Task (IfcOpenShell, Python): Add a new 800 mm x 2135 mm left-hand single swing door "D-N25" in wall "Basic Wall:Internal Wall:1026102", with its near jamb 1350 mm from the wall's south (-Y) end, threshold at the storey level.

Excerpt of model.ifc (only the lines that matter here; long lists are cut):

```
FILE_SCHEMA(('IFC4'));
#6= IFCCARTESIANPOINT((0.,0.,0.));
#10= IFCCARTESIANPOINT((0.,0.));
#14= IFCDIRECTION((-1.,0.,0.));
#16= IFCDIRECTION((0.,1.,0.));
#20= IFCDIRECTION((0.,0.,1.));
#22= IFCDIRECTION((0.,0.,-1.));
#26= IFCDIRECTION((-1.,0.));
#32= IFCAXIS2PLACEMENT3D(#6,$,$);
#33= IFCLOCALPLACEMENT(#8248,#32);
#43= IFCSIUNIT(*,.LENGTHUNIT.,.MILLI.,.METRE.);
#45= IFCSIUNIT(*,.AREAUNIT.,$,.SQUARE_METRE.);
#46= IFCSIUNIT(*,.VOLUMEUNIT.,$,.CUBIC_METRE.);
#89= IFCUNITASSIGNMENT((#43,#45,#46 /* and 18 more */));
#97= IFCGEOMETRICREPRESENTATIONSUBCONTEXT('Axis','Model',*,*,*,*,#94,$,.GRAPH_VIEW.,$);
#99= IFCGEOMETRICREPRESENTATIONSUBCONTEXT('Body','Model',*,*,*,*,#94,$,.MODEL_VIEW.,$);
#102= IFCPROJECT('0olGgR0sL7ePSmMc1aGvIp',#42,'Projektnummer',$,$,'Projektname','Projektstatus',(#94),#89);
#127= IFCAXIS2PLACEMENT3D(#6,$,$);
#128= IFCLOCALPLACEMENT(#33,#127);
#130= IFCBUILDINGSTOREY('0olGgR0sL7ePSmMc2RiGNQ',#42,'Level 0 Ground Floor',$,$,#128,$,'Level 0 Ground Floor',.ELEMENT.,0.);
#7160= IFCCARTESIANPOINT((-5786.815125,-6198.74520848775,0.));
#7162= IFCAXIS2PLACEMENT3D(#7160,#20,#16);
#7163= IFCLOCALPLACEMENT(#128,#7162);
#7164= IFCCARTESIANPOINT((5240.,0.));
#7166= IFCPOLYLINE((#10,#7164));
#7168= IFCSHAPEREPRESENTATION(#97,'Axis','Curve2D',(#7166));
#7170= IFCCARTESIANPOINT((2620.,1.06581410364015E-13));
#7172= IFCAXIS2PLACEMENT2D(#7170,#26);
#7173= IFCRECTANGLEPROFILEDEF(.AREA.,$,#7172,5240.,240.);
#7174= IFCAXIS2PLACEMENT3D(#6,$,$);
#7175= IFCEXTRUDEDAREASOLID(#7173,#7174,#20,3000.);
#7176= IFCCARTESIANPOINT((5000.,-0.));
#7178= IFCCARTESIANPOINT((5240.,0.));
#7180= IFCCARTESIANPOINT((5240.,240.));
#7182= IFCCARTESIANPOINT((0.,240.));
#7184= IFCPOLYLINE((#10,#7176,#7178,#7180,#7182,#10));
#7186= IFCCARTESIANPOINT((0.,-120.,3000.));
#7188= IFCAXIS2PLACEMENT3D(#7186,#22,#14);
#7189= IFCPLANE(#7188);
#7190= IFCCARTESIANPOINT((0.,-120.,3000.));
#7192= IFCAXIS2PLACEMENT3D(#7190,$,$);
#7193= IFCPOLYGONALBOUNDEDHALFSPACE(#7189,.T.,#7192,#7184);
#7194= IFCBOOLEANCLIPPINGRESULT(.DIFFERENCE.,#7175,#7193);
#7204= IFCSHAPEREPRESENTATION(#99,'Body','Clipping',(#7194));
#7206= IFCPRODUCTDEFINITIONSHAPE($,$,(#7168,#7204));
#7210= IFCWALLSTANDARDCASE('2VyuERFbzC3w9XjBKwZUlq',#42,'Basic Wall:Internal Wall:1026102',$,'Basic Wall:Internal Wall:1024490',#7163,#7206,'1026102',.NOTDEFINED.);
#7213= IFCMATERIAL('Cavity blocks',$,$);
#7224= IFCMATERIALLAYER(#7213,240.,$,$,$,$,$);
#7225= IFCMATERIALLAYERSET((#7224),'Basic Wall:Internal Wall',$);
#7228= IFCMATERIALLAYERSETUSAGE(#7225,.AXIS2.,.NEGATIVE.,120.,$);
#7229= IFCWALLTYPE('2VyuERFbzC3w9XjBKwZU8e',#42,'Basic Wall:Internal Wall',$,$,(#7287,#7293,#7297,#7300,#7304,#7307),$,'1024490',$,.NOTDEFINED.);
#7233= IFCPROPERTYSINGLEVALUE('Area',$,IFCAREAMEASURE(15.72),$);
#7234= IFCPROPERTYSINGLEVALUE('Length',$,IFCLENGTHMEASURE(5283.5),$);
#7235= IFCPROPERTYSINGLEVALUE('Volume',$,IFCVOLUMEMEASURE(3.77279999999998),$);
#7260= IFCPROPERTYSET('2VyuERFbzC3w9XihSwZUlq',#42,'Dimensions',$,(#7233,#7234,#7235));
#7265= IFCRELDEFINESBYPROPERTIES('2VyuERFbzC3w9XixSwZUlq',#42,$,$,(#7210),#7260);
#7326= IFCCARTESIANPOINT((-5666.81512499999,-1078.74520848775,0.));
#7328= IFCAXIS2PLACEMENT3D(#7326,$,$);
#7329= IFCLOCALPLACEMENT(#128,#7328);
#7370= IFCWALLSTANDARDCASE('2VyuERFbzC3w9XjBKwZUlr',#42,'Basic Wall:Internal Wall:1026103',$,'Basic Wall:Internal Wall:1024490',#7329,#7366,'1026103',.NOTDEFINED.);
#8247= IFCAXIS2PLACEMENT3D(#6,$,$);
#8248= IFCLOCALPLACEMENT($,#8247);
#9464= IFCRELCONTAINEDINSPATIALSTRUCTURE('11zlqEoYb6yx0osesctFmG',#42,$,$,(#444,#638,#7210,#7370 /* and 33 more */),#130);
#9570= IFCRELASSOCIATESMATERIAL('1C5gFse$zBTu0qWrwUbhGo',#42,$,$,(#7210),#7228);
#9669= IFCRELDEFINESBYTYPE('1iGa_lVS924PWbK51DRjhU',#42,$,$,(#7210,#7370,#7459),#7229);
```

```python
import numpy as np
import ifcopenshell
import ifcopenshell.api.feature
import ifcopenshell.api.geometry
import ifcopenshell.api.pset
import ifcopenshell.api.root
import ifcopenshell.api.spatial
import ifcopenshell.geom
import ifcopenshell.util.element
import ifcopenshell.util.placement
import ifcopenshell.util.representation
import ifcopenshell.util.shape
import ifcopenshell.util.unit

model = ifcopenshell.open("model.ifc")
unit_scale = ifcopenshell.util.unit.calculate_unit_scale(model)
area_scale = ifcopenshell.util.unit.calculate_unit_scale(model, "AREAUNIT")
volume_scale = ifcopenshell.util.unit.calculate_unit_scale(model, "VOLUMEUNIT")
settings = ifcopenshell.geom.settings()


def volume(element):
    """Net volume in cubic metres, openings subtracted."""
    shape = ifcopenshell.geom.create_shape(settings, element)
    return ifcopenshell.util.shape.get_volume(shape.geometry)


wall = model.by_guid("2VyuERFbzC3w9XjBKwZUlq")
storey = ifcopenshell.util.element.get_container(wall, ifc_class="IfcBuildingStorey")
context = ifcopenshell.util.representation.get_context(model, "Model", "Body", "MODEL_VIEW")
before = volume(wall)

width, height, from_end, sill = 0.8, 2.135, 1.35, 0.0  # metres

# The wall runs along its own X axis, and the end named is its -X end.
wall_shape = ifcopenshell.geom.create_shape(settings, wall)
x, y, z = ifcopenshell.util.shape.get_vertices(wall_shape.geometry).T
start = x.min() + from_end
face, thickness = float(y.min()), float(y.max() - y.min())
wall_matrix = ifcopenshell.util.placement.get_local_placement(wall.ObjectPlacement)
level = ifcopenshell.util.placement.get_local_placement(storey.ObjectPlacement)[2, 3]


def in_wall(x, y):
    """Placement at x, y metres in the wall's axes, at sill height."""
    matrix = wall_matrix.copy()
    matrix[:, 3] = wall_matrix @ np.array([x / unit_scale, y / unit_scale, 0.0, 1.0])
    matrix[2, 3] = level + sill / unit_scale
    return matrix


# Opening: a box that overshoots both wall faces by 50 mm.
opening = ifcopenshell.api.root.create_entity(model, ifc_class="IfcOpeningElement", predefined_type="OPENING")
box = ifcopenshell.api.geometry.add_wall_representation(
    model, context=context, length=width, height=height, thickness=thickness + 0.1
)
ifcopenshell.api.geometry.assign_representation(model, product=opening, representation=box)
ifcopenshell.api.geometry.edit_object_placement(model, product=opening, matrix=in_wall(start, face - 0.05), is_si=False)
ifcopenshell.api.feature.add_feature(model, feature=opening, element=wall)

door = ifcopenshell.api.root.create_entity(model, ifc_class="IfcDoor", name="D-N25", predefined_type="DOOR")
door.OverallWidth, door.OverallHeight = width / unit_scale, height / unit_scale
door.OperationType = "SINGLE_SWING_LEFT"
body = ifcopenshell.api.geometry.add_door_representation(
    model,
    context=context,
    overall_width=door.OverallWidth,
    overall_height=door.OverallHeight,
    operation_type="SINGLE_SWING_LEFT",
    lining_properties={"LiningDepth": thickness / unit_scale, "ThresholdDepth": thickness / unit_scale},
)
ifcopenshell.api.geometry.assign_representation(model, product=door, representation=body)
ifcopenshell.api.spatial.assign_container(model, products=[door], relating_structure=storey)
ifcopenshell.api.feature.add_filling(model, opening=opening, element=door)

# The lining spans the wall, so the door starts at the wall face.
ifcopenshell.api.geometry.edit_object_placement(model, product=door, matrix=in_wall(start, face), is_si=False)

after = volume(wall)

# Update the wall's stored quantities.
pset = model.by_id(ifcopenshell.util.element.get_pset(wall, "Dimensions", should_inherit=False)["id"])
ifcopenshell.api.pset.edit_pset(model, pset=pset, properties={
    "Area": model.create_entity("IfcAreaMeasure", after / thickness / area_scale),
    "Volume": model.create_entity("IfcVolumeMeasure", after / volume_scale),
})

print(f"wall volume {before:.3f} -> {after:.3f} m3")

model.write("model_v2.ifc")
```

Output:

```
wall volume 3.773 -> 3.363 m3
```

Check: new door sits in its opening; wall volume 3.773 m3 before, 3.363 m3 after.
